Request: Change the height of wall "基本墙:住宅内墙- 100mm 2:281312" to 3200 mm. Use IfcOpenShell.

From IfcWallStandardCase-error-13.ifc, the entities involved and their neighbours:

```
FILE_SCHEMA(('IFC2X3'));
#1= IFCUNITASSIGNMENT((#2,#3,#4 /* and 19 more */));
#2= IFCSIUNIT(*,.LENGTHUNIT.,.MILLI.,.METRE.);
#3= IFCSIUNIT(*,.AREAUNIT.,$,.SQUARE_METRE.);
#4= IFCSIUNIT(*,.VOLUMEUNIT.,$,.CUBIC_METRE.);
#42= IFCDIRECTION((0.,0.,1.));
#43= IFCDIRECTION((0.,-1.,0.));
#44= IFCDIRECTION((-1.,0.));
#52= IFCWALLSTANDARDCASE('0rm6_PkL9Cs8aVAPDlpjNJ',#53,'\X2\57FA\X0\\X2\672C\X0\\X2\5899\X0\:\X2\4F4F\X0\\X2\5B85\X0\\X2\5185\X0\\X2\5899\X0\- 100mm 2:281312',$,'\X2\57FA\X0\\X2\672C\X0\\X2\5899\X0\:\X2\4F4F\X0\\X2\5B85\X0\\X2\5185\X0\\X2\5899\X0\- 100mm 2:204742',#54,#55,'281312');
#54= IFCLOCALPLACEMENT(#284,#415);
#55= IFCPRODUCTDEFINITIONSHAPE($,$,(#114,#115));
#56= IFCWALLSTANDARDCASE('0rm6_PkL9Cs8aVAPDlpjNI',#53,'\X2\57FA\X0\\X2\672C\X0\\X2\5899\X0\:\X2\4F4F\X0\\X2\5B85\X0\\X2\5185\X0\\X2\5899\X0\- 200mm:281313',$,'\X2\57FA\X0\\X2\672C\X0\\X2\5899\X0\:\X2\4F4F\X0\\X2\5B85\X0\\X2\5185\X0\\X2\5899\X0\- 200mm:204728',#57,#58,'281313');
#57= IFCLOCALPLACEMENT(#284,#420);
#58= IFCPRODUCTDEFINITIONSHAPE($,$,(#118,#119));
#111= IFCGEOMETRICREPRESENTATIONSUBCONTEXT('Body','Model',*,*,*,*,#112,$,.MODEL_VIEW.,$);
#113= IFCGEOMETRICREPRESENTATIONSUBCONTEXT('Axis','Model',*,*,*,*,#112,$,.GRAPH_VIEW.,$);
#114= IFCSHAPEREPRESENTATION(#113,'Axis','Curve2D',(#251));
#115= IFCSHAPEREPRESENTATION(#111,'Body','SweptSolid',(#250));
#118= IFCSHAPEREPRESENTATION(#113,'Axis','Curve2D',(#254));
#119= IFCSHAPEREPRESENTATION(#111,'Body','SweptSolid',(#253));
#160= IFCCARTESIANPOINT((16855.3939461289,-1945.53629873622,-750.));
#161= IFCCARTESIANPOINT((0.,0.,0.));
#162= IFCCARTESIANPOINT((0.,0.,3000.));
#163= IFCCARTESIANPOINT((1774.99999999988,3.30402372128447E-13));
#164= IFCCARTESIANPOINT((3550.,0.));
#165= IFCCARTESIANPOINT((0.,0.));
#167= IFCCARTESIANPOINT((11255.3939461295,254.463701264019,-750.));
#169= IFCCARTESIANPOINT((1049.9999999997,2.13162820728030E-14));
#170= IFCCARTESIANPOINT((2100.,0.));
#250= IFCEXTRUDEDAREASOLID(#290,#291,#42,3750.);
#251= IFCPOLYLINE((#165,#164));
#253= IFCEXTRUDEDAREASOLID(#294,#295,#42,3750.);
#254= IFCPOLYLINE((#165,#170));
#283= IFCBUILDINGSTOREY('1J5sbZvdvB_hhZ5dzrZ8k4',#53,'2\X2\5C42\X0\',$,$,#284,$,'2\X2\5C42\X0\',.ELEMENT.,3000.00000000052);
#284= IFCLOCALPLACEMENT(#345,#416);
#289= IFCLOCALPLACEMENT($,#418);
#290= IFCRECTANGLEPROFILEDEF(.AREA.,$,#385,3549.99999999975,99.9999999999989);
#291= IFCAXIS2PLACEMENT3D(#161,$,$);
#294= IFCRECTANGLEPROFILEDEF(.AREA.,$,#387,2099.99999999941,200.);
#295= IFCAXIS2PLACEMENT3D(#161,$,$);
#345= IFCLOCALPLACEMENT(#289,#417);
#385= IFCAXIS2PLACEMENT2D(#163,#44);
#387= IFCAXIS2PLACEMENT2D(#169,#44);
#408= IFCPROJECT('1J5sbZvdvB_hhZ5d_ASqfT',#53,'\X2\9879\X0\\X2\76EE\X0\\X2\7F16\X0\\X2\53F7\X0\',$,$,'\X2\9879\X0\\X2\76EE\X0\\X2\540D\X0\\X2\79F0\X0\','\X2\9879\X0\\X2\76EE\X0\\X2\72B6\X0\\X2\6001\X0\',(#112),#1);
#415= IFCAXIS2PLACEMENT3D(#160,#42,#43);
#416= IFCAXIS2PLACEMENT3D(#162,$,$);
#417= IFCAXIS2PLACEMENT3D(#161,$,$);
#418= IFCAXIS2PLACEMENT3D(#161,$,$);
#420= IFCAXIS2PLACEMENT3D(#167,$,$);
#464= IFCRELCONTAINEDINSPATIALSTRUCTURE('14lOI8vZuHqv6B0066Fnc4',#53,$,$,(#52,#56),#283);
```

```python
import ifcopenshell
import ifcopenshell.geom
import ifcopenshell.util.representation
import ifcopenshell.util.shape

model = ifcopenshell.open("IfcWallStandardCase-error-13.ifc")
settings = ifcopenshell.geom.settings()


def volume(element):
    """Net volume in cubic metres, openings subtracted."""
    shape = ifcopenshell.geom.create_shape(settings, element)
    return ifcopenshell.util.shape.get_volume(shape.geometry)


wall = model.by_guid("0rm6_PkL9Cs8aVAPDlpjNJ")
before = volume(wall)

body = ifcopenshell.util.representation.get_representation(wall, "Model", "Body")
solid = body.Items[0]
old_height = solid.Depth
solid.Depth = 3200.0
after = volume(wall)

print(f"height {old_height:g} -> {solid.Depth:g}, volume {before:.3f} -> {after:.3f} m3")

model.write("IfcWallStandardCase-error-13-out.ifc")
```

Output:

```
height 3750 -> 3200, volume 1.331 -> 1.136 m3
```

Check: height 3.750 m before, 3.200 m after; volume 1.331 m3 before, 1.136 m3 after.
